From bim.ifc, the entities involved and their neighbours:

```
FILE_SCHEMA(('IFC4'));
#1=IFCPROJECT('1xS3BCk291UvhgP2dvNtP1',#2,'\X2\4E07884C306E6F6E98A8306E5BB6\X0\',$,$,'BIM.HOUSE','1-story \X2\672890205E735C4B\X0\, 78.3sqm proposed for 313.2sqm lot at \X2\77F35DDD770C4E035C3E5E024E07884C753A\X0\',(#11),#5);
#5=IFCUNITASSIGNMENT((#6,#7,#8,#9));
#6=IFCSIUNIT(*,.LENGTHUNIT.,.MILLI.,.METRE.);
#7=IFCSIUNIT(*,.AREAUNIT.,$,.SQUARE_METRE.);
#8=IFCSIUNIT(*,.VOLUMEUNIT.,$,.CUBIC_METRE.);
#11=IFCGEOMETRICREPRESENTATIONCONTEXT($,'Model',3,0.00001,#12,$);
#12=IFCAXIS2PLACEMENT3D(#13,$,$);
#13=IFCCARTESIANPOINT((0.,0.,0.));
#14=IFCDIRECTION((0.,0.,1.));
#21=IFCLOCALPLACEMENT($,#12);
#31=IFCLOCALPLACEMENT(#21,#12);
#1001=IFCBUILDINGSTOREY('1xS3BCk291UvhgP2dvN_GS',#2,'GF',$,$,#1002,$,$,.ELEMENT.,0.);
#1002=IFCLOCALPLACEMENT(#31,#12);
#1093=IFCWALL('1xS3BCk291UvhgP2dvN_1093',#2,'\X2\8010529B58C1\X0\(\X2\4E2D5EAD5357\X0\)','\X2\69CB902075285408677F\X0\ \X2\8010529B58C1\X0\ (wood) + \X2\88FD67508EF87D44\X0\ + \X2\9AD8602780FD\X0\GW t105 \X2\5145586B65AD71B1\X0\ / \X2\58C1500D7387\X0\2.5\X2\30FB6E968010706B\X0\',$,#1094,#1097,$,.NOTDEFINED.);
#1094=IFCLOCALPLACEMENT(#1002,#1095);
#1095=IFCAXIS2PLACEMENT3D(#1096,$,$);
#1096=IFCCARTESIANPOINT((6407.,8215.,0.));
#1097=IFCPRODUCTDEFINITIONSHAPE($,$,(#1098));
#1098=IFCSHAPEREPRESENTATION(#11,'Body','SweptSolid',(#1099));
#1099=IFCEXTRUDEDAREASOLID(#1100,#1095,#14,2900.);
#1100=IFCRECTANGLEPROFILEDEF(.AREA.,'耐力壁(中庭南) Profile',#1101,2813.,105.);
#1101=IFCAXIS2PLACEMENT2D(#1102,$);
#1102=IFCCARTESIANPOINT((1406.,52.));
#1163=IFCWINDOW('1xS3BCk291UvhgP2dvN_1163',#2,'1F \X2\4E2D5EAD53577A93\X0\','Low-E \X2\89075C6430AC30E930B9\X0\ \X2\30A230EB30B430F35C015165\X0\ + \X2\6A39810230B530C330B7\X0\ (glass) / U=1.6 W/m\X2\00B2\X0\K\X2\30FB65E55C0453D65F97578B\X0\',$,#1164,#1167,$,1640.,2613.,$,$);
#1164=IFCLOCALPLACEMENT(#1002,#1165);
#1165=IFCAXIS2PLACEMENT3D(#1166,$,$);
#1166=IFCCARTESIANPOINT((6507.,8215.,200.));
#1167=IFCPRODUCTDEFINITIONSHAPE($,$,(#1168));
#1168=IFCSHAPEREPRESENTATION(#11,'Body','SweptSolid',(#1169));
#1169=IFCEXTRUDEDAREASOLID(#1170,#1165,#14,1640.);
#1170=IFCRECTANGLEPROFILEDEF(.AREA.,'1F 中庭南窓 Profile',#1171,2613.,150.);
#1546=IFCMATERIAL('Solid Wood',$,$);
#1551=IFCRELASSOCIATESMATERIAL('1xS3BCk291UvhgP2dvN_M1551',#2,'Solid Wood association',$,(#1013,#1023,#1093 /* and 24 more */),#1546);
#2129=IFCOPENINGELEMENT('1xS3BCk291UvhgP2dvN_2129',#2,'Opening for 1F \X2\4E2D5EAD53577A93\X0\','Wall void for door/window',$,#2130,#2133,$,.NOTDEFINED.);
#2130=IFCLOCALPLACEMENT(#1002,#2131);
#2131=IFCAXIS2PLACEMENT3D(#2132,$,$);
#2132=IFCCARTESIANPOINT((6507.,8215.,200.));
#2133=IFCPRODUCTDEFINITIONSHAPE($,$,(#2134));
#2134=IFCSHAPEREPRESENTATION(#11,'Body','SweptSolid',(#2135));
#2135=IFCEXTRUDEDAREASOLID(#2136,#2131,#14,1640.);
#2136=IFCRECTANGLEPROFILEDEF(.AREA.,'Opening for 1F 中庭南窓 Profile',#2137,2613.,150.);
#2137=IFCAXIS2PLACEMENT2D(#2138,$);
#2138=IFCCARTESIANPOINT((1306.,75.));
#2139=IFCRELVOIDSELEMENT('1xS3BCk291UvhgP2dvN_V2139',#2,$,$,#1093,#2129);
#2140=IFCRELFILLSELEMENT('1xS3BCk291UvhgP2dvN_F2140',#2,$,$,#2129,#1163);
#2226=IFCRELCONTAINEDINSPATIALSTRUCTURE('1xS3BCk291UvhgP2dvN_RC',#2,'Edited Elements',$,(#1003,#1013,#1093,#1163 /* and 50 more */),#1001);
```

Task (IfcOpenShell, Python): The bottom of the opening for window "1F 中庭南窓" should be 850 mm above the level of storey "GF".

```python
import numpy as np
import ifcopenshell
import ifcopenshell.api.geometry
import ifcopenshell.geom
import ifcopenshell.util.element
import ifcopenshell.util.placement
import ifcopenshell.util.shape
import ifcopenshell.util.unit

model = ifcopenshell.open("bim.ifc")
unit_scale = ifcopenshell.util.unit.calculate_unit_scale(model)

window = model.by_guid("1xS3BCk291UvhgP2dvN_1163")
opening = window.FillsVoids[0].RelatingOpeningElement
storey = ifcopenshell.util.element.get_container(window, ifc_class="IfcBuildingStorey")
level = ifcopenshell.util.placement.get_local_placement(storey.ObjectPlacement)[2, 3]

# The opening's origin need not be at the sill, so measure its lowest point.
shape = ifcopenshell.geom.create_shape(ifcopenshell.geom.settings(), opening)
bottom = ifcopenshell.util.shape.get_shape_bottom_elevation(shape, shape.geometry) / unit_scale
dz = level + 0.85 / unit_scale - bottom

shift = np.array([0.0, 0.0, dz])
# The window is not placed relative to its opening, so move both.
for product in (opening, window):
    matrix = ifcopenshell.util.placement.get_local_placement(product.ObjectPlacement)
    matrix[:3, 3] += shift
    ifcopenshell.api.geometry.edit_object_placement(model, product=product, matrix=matrix, is_si=False)

print(f"moved by {dz * unit_scale:+.3f} m")

model.write("bim_v2.ifc")
```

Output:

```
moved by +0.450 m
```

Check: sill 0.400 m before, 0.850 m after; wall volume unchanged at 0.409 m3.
